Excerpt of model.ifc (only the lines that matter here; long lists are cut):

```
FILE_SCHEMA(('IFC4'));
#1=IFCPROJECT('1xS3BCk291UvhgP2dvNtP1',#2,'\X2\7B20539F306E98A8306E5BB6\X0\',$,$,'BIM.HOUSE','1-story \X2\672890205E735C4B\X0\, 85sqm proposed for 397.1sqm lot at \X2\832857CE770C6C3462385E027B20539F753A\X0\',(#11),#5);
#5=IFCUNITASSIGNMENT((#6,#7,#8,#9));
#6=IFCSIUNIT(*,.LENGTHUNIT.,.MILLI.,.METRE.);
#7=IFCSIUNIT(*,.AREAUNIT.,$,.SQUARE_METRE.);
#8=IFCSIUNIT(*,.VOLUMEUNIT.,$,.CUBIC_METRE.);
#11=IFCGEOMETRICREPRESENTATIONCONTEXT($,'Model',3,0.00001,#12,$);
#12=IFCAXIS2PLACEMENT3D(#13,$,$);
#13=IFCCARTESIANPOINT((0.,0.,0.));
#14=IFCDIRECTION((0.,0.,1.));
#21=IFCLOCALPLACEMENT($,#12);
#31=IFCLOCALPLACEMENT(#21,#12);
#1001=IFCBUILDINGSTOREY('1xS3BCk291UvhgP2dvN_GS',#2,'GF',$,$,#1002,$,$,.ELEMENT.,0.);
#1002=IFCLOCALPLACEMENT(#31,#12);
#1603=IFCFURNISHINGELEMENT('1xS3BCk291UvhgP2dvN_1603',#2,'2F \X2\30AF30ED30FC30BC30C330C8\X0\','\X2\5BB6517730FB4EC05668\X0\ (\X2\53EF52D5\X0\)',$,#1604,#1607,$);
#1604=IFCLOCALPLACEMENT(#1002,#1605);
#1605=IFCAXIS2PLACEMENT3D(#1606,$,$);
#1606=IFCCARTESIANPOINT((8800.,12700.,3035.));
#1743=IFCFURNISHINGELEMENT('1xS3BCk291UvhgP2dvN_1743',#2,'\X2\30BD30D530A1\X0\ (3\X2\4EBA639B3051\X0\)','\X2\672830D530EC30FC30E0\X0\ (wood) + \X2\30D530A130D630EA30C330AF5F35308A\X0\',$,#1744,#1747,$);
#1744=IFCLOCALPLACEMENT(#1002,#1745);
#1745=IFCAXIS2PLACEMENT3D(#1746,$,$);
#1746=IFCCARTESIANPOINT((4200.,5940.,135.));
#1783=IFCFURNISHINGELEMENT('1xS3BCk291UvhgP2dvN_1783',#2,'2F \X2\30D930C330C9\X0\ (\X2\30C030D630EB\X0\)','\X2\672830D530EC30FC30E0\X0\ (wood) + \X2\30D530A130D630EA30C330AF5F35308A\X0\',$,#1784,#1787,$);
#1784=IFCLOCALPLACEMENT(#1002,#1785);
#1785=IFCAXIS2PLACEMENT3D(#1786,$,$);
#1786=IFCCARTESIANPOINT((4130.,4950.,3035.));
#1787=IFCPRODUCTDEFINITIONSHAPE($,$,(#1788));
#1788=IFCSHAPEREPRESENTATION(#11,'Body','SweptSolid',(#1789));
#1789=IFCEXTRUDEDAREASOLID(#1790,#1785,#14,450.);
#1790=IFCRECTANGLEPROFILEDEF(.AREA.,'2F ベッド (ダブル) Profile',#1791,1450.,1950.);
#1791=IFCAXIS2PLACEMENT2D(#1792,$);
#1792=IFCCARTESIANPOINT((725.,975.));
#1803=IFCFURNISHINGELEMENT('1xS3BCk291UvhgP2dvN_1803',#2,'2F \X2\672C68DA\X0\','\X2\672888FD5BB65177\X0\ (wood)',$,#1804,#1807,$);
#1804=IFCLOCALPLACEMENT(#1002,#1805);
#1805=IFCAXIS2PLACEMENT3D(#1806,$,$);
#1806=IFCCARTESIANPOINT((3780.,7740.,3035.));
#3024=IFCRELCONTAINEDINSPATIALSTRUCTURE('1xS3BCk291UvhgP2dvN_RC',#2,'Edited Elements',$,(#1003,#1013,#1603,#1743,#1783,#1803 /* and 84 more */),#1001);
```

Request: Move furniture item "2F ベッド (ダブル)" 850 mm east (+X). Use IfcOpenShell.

```python
import ifcopenshell
import ifcopenshell.api.geometry
import ifcopenshell.util.placement

model = ifcopenshell.open("model.ifc")

item = model.by_id(1783)
matrix = ifcopenshell.util.placement.get_local_placement(item.ObjectPlacement)
matrix[0, 3] += 850.0
ifcopenshell.api.geometry.edit_object_placement(model, product=item, matrix=matrix, is_si=False)

print(ifcopenshell.util.placement.get_local_placement(item.ObjectPlacement).round(3) + 0.0)

model.write("model_v2.ifc")
```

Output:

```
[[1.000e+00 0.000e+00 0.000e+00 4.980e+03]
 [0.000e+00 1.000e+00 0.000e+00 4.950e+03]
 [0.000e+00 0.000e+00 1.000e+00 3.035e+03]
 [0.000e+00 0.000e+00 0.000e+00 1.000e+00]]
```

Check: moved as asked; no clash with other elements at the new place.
